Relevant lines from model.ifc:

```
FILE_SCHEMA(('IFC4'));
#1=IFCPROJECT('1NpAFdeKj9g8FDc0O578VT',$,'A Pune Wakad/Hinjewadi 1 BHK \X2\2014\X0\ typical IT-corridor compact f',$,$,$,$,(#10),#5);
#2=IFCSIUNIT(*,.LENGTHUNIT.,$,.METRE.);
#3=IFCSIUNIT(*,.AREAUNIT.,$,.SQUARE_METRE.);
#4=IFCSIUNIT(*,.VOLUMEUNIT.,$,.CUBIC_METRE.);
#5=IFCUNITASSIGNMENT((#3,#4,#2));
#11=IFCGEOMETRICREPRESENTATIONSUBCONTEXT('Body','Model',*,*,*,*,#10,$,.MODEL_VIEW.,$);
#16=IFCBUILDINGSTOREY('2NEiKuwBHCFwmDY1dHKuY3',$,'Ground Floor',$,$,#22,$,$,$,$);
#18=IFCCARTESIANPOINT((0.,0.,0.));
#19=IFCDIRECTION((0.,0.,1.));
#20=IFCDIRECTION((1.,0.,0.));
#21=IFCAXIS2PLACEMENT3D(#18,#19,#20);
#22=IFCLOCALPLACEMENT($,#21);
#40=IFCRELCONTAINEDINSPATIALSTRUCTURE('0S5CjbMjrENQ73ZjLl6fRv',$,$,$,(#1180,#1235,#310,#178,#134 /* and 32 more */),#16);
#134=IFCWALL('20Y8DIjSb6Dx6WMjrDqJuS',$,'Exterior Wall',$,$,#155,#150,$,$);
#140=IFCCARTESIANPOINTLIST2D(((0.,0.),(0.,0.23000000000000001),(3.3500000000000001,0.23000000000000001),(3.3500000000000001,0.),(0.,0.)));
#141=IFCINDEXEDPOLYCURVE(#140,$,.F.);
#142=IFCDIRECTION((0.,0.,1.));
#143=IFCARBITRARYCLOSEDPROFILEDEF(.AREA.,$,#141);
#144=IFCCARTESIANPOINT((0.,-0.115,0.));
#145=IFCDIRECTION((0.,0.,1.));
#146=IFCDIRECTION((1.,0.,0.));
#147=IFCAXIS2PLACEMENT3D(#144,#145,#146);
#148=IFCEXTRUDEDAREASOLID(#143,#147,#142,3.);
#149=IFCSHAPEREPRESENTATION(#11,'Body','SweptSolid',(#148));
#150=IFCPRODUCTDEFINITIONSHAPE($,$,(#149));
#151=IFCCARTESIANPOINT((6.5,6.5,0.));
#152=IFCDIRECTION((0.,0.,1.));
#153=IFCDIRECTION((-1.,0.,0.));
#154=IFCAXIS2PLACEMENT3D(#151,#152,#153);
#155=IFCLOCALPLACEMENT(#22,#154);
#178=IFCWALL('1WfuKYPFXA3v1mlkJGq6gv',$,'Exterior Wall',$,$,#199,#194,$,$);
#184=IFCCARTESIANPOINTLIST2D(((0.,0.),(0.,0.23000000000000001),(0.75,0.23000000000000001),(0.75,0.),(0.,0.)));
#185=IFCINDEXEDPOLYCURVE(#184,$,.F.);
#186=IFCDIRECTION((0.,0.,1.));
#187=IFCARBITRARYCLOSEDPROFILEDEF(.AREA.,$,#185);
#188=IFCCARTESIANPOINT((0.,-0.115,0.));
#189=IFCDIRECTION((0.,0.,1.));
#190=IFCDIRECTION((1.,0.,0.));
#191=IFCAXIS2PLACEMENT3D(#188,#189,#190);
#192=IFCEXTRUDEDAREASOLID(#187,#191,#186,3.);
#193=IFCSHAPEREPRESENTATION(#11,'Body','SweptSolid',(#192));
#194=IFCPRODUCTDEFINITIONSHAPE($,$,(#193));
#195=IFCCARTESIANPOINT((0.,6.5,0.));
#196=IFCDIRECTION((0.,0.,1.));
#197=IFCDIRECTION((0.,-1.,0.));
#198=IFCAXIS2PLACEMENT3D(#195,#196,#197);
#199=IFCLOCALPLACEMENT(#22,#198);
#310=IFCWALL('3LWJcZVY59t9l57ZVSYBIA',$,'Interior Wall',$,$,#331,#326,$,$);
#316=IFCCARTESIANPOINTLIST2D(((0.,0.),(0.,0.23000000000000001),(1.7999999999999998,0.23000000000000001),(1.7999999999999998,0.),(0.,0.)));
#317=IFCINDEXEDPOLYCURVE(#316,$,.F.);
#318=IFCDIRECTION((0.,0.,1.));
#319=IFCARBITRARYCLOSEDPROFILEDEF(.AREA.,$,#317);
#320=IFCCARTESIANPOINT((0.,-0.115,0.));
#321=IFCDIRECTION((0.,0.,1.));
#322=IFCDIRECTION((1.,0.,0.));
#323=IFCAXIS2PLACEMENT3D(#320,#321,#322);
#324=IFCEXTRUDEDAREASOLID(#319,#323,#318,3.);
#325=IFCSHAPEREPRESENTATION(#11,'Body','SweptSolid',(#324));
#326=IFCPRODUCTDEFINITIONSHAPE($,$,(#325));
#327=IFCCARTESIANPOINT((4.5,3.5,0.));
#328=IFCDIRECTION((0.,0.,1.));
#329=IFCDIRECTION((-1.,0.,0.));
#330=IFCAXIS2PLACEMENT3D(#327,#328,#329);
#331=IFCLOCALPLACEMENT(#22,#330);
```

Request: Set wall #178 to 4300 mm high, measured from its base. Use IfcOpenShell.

```python
import ifcopenshell
import ifcopenshell.geom
import ifcopenshell.util.representation
import ifcopenshell.util.shape

model = ifcopenshell.open("model.ifc")
settings = ifcopenshell.geom.settings()


def volume(element):
    """Net volume in cubic metres, openings subtracted."""
    shape = ifcopenshell.geom.create_shape(settings, element)
    return ifcopenshell.util.shape.get_volume(shape.geometry)


wall = model.by_id(178)
before = volume(wall)

body = ifcopenshell.util.representation.get_representation(wall, "Model", "Body")
solid = body.Items[0]
old_height = solid.Depth
solid.Depth = 4.3
after = volume(wall)

print(f"height {old_height:g} -> {solid.Depth:g}, volume {before:.3f} -> {after:.3f} m3")

model.write("model_v2.ifc")
```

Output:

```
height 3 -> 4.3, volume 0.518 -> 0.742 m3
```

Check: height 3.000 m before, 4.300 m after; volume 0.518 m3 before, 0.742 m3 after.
